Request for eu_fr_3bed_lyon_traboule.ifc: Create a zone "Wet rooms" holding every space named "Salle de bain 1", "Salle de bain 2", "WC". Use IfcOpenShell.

First a look at what the model holds.

```python
import ifcopenshell

model = ifcopenshell.open("eu_fr_3bed_lyon_traboule.ifc")
print(model.schema)
seen = {}
for space in model.by_type("IfcSpace"):
    seen[space.LongName] = seen.get(space.LongName, 0) + 1
for name, count in sorted(seen.items(), key=str):
    print(count, "x", name)
print("zones:", [z.Name for z in model.by_type("IfcZone")][:20])
```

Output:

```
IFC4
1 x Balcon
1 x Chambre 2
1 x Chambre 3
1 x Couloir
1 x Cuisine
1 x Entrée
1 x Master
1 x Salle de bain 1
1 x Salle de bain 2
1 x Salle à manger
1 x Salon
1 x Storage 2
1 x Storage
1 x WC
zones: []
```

```python
import ifcopenshell
import ifcopenshell.api.group
import ifcopenshell.api.root

model = ifcopenshell.open("eu_fr_3bed_lyon_traboule.ifc")

names = {"Salle de bain 1", "Salle de bain 2", "WC"}
spaces = [s for s in model.by_type("IfcSpace") if s.LongName in names]

zone = ifcopenshell.api.root.create_entity(model, ifc_class="IfcZone", name="Wet rooms")
ifcopenshell.api.group.assign_group(model, products=spaces, group=zone)
print(len(spaces), "spaces in", zone.Name)

model.write("eu_fr_3bed_lyon_traboule-out.ifc")
```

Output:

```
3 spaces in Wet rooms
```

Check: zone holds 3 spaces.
